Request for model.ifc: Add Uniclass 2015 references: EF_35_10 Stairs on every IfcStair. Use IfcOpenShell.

First a look at what the model holds.

```python
import ifcopenshell

model = ifcopenshell.open("model.ifc")
print(model.schema)
print("classifications:", [c.Name for c in model.by_type("IfcClassification")])
for ifc_class in ("IfcDoor", "IfcRoof", "IfcStair", "IfcWall", "IfcWindow"):
    print(ifc_class, len(model.by_type(ifc_class)))
```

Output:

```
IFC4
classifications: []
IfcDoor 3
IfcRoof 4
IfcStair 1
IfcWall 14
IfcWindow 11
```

```python
import ifcopenshell
import ifcopenshell.api.classification

model = ifcopenshell.open("model.ifc")

system = ifcopenshell.api.classification.add_classification(model, classification="Uniclass 2015")

codes = {
    "IfcStair": ("EF_35_10", "Stairs"),
}
for ifc_class, (code, name) in codes.items():
    products = model.by_type(ifc_class)
    ifcopenshell.api.classification.add_reference(
        model, products=products, classification=system, identification=code, name=name
    )
    print(code, len(products))

model.write("model-out.ifc")
```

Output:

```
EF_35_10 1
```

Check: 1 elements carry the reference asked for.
